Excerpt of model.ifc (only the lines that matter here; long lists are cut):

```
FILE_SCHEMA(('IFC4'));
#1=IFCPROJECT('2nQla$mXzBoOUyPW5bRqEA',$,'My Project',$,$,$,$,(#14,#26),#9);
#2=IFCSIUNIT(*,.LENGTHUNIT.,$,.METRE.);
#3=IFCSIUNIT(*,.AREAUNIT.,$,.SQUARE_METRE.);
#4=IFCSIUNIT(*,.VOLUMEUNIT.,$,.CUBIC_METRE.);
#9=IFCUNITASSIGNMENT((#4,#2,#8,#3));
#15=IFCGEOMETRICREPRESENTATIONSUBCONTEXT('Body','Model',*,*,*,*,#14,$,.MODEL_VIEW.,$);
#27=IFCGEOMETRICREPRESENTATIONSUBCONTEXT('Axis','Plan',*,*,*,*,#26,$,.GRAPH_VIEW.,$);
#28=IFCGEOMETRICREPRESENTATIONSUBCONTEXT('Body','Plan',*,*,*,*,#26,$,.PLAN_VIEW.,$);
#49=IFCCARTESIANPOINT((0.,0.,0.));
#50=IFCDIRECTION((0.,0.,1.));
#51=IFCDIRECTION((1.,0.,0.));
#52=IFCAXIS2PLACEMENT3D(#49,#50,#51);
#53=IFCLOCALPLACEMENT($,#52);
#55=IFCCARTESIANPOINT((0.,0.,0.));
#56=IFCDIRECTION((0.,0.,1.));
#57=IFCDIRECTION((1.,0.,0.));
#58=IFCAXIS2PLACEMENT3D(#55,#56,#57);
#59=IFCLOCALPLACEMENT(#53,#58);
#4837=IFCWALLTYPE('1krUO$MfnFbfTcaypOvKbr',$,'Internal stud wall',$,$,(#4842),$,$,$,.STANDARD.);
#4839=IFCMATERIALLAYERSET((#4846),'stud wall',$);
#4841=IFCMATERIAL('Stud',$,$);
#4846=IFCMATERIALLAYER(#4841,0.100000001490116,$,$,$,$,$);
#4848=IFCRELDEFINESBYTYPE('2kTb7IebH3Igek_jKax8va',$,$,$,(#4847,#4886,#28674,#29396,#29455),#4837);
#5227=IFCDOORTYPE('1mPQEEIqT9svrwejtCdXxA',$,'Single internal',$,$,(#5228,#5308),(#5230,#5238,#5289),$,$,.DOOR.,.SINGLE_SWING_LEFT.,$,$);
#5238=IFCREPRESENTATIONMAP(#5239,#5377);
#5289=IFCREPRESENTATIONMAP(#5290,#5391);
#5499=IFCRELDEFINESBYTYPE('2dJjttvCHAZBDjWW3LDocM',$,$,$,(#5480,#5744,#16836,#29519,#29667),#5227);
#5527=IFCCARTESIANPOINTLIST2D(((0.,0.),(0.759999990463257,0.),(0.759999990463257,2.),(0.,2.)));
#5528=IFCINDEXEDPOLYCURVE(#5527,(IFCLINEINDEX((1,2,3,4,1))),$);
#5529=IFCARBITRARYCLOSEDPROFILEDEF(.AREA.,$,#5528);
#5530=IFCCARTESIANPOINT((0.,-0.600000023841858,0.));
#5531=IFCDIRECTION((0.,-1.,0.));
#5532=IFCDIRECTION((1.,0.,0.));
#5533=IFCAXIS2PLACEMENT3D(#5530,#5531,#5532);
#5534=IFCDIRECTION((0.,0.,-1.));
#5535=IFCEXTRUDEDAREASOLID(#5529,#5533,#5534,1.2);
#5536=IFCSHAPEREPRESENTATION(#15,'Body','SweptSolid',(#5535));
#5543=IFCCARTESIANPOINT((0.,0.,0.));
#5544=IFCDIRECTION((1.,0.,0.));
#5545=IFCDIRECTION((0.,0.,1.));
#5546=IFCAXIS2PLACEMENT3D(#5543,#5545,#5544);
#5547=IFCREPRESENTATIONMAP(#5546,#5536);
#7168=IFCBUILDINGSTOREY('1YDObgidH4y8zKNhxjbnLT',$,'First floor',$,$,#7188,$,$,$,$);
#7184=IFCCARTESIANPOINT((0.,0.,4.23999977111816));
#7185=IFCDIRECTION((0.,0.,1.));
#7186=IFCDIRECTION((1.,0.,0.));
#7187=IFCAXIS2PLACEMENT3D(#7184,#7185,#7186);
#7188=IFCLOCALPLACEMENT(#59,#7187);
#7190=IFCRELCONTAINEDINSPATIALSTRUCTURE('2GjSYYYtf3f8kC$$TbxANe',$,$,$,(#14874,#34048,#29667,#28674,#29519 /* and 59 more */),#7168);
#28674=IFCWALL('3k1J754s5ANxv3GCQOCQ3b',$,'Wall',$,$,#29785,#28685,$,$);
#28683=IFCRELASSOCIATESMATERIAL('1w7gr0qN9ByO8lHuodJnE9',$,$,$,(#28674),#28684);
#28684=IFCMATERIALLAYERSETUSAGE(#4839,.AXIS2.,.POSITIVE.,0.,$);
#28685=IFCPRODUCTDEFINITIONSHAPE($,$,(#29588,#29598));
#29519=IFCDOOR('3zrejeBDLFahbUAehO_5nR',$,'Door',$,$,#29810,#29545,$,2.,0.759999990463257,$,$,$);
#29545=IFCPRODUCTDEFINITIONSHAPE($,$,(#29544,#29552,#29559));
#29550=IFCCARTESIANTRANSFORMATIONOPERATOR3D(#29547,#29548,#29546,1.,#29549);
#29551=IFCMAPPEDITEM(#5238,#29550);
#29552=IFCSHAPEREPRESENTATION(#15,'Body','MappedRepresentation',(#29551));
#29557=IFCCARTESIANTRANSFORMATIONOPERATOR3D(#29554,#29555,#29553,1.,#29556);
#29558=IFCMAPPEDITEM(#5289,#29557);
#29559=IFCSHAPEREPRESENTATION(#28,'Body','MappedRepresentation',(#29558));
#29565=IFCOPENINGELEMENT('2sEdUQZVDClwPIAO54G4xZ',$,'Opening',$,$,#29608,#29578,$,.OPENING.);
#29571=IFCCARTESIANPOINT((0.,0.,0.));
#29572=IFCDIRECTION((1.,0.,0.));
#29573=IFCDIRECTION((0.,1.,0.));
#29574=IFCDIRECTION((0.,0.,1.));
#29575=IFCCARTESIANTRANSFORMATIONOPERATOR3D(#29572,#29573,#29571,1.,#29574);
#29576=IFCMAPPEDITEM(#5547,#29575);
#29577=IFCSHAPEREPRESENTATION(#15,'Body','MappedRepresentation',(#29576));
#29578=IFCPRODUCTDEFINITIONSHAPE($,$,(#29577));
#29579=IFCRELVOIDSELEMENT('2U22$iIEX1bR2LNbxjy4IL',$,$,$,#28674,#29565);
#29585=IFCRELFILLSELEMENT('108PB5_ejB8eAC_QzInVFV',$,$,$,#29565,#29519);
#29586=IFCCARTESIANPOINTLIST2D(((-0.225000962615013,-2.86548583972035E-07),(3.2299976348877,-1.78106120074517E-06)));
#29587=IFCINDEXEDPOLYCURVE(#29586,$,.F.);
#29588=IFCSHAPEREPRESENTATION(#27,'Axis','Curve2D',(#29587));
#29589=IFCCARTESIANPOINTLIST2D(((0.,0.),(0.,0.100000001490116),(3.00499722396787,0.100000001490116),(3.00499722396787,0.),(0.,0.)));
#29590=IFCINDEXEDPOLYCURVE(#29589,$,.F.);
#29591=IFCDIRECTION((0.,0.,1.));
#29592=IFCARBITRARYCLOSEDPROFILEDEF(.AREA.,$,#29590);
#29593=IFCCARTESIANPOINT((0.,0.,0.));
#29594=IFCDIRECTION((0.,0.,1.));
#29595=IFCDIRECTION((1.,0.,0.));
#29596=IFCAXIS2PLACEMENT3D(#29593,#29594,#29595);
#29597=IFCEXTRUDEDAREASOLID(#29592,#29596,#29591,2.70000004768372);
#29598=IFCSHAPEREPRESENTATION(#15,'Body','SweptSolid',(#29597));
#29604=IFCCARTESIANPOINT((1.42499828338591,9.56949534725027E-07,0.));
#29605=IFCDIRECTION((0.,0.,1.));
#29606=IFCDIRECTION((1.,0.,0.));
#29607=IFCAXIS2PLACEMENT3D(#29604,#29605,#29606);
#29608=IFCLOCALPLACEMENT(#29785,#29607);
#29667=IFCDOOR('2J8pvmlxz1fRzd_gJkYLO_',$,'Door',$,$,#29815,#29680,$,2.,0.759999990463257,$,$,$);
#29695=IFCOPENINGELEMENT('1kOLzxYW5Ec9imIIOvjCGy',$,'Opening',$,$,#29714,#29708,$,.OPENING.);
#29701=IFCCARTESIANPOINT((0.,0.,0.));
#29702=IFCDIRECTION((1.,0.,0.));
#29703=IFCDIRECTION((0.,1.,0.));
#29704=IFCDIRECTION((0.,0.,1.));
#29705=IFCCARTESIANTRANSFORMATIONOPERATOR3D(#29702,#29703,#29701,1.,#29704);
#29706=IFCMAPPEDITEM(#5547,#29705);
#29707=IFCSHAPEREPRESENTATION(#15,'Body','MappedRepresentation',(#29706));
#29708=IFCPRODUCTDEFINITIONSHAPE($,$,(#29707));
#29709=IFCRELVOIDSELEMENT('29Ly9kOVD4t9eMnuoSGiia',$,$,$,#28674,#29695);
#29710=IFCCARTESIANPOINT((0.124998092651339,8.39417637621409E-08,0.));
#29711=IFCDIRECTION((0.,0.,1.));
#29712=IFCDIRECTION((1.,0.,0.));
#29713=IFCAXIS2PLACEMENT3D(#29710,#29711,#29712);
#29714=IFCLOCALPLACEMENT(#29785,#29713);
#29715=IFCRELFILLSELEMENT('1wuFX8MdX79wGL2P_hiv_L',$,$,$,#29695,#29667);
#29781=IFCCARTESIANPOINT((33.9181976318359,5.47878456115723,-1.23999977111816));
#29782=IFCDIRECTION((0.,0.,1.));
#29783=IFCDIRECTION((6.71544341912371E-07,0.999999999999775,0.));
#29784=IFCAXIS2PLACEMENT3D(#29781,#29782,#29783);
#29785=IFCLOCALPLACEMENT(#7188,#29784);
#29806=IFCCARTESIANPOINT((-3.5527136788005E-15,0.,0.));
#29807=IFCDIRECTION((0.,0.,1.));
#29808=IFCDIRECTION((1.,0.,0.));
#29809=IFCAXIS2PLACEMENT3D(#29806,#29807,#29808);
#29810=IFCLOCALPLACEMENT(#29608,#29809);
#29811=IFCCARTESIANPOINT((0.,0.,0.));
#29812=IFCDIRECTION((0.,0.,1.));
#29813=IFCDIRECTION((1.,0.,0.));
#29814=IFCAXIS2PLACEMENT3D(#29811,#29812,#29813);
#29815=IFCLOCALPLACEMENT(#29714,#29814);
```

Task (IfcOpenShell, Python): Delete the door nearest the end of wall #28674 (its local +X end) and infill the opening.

```python
import ifcopenshell
import ifcopenshell.api.feature
import ifcopenshell.api.root
import ifcopenshell.geom
import ifcopenshell.util.shape

model = ifcopenshell.open("model.ifc")
settings = ifcopenshell.geom.settings()


def volume(element):
    """Net volume in cubic metres, openings subtracted."""
    shape = ifcopenshell.geom.create_shape(settings, element)
    return ifcopenshell.util.shape.get_volume(shape.geometry)


door = model.by_id(29519)
opening = door.FillsVoids[0].RelatingOpeningElement
wall = opening.VoidsElements[0].RelatingBuildingElement
before = volume(wall)

ifcopenshell.api.root.remove_product(model, product=door)
ifcopenshell.api.feature.remove_feature(model, feature=opening)

after = volume(wall)

print(f"wall volume {before:.3f} -> {after:.3f} m3")

model.write("model_updated.ifc")
```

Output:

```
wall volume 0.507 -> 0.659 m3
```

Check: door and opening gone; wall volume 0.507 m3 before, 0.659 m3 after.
